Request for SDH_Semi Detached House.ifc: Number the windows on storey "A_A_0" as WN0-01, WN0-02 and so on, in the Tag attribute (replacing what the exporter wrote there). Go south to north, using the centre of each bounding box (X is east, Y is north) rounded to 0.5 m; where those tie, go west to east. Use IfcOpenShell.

First a look at what the model holds.

```python
import ifcopenshell
import ifcopenshell.util.element
import ifcopenshell.util.placement

model = ifcopenshell.open("SDH_Semi Detached House.ifc")
print(model.schema)
storey = next(s for s in model.by_type("IfcBuildingStorey") if s.Name == "A_A_0")
windows = [e for e in ifcopenshell.util.element.get_decomposition(storey) if e.is_a("IfcWindow")]
for e in sorted(windows, key=lambda e: e.id()):
    origin = ifcopenshell.util.placement.get_local_placement(e.ObjectPlacement)[:3, 3]
    print(e.id(), e.Tag, e.Name, origin.round(2) + 0.0, sep=" | ")
```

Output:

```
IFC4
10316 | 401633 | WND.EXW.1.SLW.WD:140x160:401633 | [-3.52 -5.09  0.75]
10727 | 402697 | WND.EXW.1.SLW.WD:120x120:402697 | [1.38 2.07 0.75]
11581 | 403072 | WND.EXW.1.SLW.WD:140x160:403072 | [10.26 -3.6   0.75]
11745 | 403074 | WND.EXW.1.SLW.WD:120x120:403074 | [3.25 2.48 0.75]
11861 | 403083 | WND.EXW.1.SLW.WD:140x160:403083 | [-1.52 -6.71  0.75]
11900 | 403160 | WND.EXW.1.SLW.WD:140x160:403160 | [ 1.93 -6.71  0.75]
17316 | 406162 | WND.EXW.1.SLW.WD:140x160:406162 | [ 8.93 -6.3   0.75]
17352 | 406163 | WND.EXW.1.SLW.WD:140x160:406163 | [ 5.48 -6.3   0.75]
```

```python
import ifcopenshell
import ifcopenshell.geom
import ifcopenshell.util.element
import ifcopenshell.util.shape

model = ifcopenshell.open("SDH_Semi Detached House.ifc")
settings = ifcopenshell.geom.settings()
settings.set("use-world-coords", True)


def centre(element):
    shape = ifcopenshell.geom.create_shape(settings, element)
    return ifcopenshell.util.shape.get_bbox_centroid(shape.geometry)


storey = next(s for s in model.by_type("IfcBuildingStorey") if s.Name == "A_A_0")
windows = [e for e in ifcopenshell.util.element.get_decomposition(storey) if e.is_a("IfcWindow")]

# Insertion points can sit at a corner or the storey origin, so sort by the geometry (in metres).
centres = {e: centre(e) for e in windows}
windows.sort(key=lambda e: (round(centres[e][1] / 0.5), centres[e][0]))

for i, e in enumerate(windows, start=1):
    number = f"WN0-{i:02d}"
    e.Tag = number
    print(e.id(), number)

model.write("SDH_Semi Detached House_v2.ifc")
```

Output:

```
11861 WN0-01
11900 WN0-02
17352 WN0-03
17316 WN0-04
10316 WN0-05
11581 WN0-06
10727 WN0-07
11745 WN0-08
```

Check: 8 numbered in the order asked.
